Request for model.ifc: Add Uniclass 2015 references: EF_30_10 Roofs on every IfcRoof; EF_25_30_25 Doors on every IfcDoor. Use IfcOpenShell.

First a look at what the model holds.

```python
import ifcopenshell

model = ifcopenshell.open("model.ifc")
print(model.schema)
print("classifications:", [c.Name for c in model.by_type("IfcClassification")])
for ifc_class in ("IfcDoor", "IfcRoof", "IfcStair", "IfcWall", "IfcWindow"):
    print(ifc_class, len(model.by_type(ifc_class)))
```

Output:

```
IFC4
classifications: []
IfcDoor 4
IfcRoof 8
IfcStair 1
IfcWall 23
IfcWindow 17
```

```python
import ifcopenshell
import ifcopenshell.api.classification

model = ifcopenshell.open("model.ifc")

system = ifcopenshell.api.classification.add_classification(model, classification="Uniclass 2015")

codes = {
    "IfcRoof": ("EF_30_10", "Roofs"),
    "IfcDoor": ("EF_25_30_25", "Doors"),
}
for ifc_class, (code, name) in codes.items():
    products = model.by_type(ifc_class)
    ifcopenshell.api.classification.add_reference(
        model, products=products, classification=system, identification=code, name=name
    )
    print(code, len(products))

model.write("model_edited.ifc")
```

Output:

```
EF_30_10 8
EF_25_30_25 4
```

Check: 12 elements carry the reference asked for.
